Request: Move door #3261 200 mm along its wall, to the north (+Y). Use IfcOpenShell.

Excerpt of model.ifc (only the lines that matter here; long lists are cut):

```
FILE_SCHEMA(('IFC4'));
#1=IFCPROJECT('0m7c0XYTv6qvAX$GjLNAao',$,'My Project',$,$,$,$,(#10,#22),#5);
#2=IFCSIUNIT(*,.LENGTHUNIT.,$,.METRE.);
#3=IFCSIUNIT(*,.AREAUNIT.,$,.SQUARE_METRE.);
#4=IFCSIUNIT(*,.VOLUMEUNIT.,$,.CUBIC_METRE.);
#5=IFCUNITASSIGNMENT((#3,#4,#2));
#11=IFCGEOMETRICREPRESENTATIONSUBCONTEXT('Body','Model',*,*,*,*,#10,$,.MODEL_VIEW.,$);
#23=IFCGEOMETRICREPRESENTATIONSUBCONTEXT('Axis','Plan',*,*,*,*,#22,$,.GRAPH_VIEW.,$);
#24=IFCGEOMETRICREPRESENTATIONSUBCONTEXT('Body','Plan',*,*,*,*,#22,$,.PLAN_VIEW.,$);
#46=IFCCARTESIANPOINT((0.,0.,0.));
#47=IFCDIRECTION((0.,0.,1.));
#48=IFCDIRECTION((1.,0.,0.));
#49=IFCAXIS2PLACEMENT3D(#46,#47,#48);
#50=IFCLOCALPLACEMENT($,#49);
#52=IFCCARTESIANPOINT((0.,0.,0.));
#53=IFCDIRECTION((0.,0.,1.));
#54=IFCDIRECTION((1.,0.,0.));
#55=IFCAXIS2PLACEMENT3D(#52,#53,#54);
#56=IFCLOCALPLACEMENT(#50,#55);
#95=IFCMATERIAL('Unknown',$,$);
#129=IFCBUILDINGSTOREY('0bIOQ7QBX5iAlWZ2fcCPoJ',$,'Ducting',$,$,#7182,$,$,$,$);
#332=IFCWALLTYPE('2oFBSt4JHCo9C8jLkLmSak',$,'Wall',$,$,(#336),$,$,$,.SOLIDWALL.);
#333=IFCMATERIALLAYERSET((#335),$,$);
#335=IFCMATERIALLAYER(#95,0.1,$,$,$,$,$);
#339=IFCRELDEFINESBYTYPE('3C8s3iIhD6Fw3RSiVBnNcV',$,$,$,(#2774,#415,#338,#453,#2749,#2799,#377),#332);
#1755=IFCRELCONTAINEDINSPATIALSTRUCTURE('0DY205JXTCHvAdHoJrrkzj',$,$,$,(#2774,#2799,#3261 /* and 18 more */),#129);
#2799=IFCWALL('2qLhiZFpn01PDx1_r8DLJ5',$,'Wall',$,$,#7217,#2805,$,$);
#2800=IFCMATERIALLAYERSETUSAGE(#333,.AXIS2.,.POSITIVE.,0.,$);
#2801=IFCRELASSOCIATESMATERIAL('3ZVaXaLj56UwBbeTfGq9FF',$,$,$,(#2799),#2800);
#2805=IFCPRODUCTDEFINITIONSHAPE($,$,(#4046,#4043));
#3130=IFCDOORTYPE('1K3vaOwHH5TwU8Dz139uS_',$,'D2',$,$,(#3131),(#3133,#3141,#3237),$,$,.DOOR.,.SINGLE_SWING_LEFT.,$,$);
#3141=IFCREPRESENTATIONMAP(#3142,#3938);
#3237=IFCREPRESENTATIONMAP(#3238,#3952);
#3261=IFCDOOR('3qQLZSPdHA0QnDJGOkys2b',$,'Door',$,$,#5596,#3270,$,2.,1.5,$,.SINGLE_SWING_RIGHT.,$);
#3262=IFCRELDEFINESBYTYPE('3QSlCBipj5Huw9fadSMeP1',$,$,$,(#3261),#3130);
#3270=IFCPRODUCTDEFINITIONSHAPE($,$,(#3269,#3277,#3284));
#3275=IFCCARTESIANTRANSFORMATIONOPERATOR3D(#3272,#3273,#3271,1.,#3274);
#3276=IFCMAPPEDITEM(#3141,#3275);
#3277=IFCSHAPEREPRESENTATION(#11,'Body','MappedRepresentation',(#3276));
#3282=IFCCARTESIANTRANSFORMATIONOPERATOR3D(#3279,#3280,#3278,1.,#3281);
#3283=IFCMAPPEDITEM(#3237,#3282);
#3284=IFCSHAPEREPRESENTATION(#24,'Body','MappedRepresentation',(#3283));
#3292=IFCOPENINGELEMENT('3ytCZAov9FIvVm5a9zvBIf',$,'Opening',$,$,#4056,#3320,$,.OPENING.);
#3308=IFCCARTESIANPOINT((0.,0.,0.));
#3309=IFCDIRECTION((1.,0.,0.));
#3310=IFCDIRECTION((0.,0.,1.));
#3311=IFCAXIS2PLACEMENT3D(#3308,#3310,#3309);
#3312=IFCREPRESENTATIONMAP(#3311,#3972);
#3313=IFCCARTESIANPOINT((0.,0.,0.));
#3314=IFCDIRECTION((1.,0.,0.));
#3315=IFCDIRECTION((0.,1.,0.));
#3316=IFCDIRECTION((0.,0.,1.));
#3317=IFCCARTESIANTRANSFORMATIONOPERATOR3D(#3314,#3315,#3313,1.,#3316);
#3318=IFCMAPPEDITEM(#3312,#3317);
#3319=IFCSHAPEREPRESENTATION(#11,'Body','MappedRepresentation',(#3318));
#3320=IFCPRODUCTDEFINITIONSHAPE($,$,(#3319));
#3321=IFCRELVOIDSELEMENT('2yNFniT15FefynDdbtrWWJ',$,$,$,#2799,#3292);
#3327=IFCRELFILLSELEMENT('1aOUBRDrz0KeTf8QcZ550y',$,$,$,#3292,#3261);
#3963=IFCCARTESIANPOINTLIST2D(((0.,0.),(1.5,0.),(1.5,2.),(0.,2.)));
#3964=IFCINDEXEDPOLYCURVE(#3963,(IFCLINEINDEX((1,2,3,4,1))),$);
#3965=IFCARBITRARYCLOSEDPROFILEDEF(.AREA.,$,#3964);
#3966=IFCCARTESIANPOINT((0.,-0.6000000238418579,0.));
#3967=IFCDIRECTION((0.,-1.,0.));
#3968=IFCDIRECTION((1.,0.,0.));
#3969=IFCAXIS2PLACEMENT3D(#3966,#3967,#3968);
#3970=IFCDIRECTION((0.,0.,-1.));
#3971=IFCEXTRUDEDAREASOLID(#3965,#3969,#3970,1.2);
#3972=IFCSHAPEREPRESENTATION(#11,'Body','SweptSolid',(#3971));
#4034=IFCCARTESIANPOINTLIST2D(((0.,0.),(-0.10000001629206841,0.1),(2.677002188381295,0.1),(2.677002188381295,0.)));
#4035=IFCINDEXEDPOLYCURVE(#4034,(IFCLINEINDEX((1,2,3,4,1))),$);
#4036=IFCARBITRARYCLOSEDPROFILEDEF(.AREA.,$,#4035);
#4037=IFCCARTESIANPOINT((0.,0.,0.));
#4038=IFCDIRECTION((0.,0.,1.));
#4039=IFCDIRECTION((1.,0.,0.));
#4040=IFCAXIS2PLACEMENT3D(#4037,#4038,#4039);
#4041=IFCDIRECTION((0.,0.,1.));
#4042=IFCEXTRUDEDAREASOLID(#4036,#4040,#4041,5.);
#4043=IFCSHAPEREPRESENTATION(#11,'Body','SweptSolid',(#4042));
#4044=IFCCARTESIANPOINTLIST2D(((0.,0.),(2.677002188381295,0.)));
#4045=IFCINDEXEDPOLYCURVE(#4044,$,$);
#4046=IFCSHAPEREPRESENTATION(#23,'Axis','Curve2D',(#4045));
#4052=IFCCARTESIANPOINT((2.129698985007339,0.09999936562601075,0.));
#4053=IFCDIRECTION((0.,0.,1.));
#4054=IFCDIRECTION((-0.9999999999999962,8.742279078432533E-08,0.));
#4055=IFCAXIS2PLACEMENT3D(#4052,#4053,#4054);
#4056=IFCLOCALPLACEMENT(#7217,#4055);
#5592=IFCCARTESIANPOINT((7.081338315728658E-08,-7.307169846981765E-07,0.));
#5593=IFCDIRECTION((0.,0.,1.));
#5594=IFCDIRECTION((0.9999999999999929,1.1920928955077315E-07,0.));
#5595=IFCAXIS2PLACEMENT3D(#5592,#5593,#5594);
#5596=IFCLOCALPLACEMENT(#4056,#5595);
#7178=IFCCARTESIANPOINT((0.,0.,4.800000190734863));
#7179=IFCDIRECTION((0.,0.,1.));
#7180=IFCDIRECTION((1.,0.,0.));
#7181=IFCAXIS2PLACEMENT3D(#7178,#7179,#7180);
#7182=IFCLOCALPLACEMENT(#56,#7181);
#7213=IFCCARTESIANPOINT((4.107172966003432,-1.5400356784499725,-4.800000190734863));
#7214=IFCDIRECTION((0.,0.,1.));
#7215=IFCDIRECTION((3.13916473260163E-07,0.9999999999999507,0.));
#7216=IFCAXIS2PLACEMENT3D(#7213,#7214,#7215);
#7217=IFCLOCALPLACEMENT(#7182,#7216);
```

```python
import ifcopenshell
import ifcopenshell.api.geometry
import ifcopenshell.util.placement

model = ifcopenshell.open("model.ifc")

door = model.by_id(3261)
opening = door.FillsVoids[0].RelatingOpeningElement
wall = opening.VoidsElements[0].RelatingBuildingElement

wall_matrix = ifcopenshell.util.placement.get_local_placement(wall.ObjectPlacement)
shift = wall_matrix[:3, 0] * 0.2
before = ifcopenshell.util.placement.get_local_placement(door.ObjectPlacement)[:3, 3].copy()

# The door is placed relative to its opening, so it follows when the opening moves.
matrix = ifcopenshell.util.placement.get_local_placement(opening.ObjectPlacement)
matrix[:3, 3] += shift
ifcopenshell.api.geometry.edit_object_placement(
    model, product=opening, matrix=matrix, is_si=False, should_transform_children=True
)

after = ifcopenshell.util.placement.get_local_placement(door.ObjectPlacement)[:3, 3]
print("door moved by", (after - before).round(3) + 0.0)

model.write("model_rev.ifc")
```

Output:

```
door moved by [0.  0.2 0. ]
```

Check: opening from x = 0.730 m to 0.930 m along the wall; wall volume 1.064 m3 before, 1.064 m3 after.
